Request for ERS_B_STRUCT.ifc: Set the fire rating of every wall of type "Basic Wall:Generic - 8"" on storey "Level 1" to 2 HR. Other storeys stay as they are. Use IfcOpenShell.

First a look at what the model holds.

```python
import ifcopenshell
import ifcopenshell.util.element

model = ifcopenshell.open("ERS_B_STRUCT.ifc")
print(model.schema)
storey = next(s for s in model.by_type("IfcBuildingStorey") if s.Name == "Level 1")
walls = [e for e in ifcopenshell.util.element.get_decomposition(storey) if e.is_a("IfcWall")]
seen = {}
for e in walls:
    element_type = ifcopenshell.util.element.get_type(e)
    key = (element_type.Name if element_type != e and element_type else None, ifcopenshell.util.element.get_pset(e, "Pset_WallCommon", "FireRating"))
    seen[key] = seen.get(key, 0) + 1
for (name, value), count in sorted(seen.items(), key=str):
    print(count, "x", name, "|", value)
```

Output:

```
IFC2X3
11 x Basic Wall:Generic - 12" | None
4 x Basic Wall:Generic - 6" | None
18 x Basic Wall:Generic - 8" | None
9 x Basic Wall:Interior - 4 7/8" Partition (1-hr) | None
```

```python
import ifcopenshell
import ifcopenshell.api.pset
import ifcopenshell.util.element

model = ifcopenshell.open("ERS_B_STRUCT.ifc")

storey = next(s for s in model.by_type("IfcBuildingStorey") if s.Name == "Level 1")
walls = [e for e in ifcopenshell.util.element.get_decomposition(storey) if e.is_a("IfcWall")]

count = 0
for e in walls:
    element_type = ifcopenshell.util.element.get_type(e)
    if element_type in (None, e) or element_type.Name != 'Basic Wall:Generic - 8"':
        continue
    # add_pset returns the element's existing set when there is one.
    pset = ifcopenshell.api.pset.add_pset(model, product=e, name="Pset_WallCommon")
    ifcopenshell.api.pset.edit_pset(model, pset=pset, properties={"FireRating": "2 HR"})
    count += 1

print(count, "walls updated")

model.write("ERS_B_STRUCT_edited.ifc")
```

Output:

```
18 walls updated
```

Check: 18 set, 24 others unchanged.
